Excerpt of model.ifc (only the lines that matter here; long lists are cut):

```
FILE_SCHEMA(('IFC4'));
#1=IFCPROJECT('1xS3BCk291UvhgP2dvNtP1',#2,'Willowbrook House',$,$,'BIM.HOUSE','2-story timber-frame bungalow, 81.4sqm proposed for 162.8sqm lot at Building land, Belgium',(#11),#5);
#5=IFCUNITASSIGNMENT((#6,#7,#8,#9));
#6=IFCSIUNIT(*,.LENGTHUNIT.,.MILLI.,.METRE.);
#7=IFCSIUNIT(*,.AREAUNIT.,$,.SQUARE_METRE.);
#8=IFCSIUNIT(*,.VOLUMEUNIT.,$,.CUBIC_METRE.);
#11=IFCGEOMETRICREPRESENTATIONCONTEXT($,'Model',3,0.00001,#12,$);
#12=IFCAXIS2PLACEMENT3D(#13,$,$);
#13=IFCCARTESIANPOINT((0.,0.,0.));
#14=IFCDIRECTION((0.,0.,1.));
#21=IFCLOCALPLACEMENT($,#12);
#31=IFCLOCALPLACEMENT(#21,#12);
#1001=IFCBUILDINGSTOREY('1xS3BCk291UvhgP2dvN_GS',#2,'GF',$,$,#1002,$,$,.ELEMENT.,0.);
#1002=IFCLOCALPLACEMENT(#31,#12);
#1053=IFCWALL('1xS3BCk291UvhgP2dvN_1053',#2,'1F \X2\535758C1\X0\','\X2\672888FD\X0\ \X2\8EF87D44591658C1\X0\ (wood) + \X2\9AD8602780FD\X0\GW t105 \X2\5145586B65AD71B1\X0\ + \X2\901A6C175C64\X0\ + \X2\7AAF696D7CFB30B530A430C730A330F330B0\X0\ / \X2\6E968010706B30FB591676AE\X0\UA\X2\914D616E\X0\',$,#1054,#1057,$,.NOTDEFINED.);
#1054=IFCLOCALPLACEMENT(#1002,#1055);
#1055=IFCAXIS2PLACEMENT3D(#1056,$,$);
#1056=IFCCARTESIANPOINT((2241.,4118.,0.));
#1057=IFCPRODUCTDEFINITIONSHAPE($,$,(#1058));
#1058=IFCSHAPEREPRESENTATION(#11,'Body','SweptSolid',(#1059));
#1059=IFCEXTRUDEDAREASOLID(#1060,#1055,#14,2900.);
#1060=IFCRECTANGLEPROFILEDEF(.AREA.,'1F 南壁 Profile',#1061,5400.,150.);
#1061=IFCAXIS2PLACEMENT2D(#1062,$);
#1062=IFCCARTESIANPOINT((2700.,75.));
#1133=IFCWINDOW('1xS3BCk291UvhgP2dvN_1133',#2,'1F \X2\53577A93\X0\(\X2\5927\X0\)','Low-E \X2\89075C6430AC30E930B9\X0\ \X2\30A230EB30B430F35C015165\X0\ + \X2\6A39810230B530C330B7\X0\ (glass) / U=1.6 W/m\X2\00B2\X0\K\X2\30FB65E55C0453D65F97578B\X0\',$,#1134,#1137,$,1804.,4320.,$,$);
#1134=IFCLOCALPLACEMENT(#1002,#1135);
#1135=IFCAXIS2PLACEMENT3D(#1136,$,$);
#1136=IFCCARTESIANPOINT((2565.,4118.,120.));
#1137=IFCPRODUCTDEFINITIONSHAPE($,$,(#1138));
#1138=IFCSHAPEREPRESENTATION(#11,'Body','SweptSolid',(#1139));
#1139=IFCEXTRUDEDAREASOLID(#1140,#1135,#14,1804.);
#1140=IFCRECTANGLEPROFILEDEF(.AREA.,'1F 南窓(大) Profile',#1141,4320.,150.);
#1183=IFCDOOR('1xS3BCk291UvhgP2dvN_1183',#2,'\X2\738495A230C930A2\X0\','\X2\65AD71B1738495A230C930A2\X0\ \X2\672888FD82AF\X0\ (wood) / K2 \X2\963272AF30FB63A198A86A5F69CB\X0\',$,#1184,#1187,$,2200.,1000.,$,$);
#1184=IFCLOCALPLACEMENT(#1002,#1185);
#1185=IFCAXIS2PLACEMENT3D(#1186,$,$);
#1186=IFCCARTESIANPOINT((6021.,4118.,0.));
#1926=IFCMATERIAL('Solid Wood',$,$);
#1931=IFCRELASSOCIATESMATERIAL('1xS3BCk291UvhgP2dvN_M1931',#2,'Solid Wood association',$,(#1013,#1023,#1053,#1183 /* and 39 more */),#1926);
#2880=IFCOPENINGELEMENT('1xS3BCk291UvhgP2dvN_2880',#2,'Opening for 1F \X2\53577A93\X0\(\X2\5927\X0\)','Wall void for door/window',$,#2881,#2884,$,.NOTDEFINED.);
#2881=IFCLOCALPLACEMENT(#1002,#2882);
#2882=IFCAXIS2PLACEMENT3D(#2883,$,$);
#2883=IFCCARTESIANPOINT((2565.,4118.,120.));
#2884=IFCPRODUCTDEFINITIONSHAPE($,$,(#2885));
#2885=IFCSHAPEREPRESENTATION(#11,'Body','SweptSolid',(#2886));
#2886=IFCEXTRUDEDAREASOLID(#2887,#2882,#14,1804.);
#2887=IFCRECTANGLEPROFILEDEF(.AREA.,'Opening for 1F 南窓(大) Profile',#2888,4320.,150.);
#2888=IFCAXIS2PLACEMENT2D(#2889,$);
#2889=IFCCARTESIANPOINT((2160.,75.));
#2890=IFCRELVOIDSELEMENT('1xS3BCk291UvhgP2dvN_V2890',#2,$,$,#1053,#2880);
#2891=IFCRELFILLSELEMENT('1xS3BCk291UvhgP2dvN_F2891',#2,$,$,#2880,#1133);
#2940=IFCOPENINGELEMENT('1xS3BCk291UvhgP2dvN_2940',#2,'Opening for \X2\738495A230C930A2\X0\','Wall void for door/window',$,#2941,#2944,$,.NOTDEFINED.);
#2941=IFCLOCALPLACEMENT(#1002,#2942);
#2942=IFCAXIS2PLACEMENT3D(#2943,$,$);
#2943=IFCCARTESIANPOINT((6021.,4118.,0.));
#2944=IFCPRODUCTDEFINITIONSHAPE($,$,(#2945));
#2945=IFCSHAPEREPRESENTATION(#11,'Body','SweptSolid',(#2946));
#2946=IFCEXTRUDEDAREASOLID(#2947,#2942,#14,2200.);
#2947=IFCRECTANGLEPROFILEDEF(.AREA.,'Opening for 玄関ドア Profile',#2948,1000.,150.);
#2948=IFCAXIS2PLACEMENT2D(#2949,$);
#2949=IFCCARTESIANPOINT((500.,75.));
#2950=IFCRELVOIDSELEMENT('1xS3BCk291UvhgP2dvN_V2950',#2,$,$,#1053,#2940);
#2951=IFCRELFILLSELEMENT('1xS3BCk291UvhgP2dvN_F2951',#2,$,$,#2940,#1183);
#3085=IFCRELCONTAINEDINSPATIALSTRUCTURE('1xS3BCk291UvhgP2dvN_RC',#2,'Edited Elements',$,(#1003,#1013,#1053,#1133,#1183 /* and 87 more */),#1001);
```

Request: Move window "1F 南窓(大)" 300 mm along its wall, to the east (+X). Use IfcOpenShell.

```python
import ifcopenshell
import ifcopenshell.api.geometry
import ifcopenshell.util.placement

model = ifcopenshell.open("model.ifc")

window = model.by_id(1133)
opening = window.FillsVoids[0].RelatingOpeningElement
wall = opening.VoidsElements[0].RelatingBuildingElement

wall_matrix = ifcopenshell.util.placement.get_local_placement(wall.ObjectPlacement)
shift = wall_matrix[:3, 0] * 300.0
before = ifcopenshell.util.placement.get_local_placement(window.ObjectPlacement)[:3, 3].copy()

# The window is not placed relative to its opening, so move both.
for product in (opening, window):
    matrix = ifcopenshell.util.placement.get_local_placement(product.ObjectPlacement)
    matrix[:3, 3] += shift
    ifcopenshell.api.geometry.edit_object_placement(model, product=product, matrix=matrix, is_si=False)

after = ifcopenshell.util.placement.get_local_placement(window.ObjectPlacement)[:3, 3]
print("window moved by", (after - before).round(3) + 0.0)

model.write("model_v2.ifc")
```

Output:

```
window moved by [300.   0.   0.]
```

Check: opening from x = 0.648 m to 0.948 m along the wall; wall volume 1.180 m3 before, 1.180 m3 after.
